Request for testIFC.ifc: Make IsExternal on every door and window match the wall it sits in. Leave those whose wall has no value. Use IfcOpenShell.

First a look at what the model holds.

```python
import ifcopenshell
import ifcopenshell.util.element

model = ifcopenshell.open("testIFC.ifc")
print(model.schema)
seen = {}
for e in model.by_type("IfcDoor") + model.by_type("IfcWindow"):
    if not e.FillsVoids:
        continue
    host = e.FillsVoids[0].RelatingOpeningElement.VoidsElements[0].RelatingBuildingElement
    own = ifcopenshell.util.element.get_pset(e, f"Pset_{e.is_a()[3:].removesuffix('StandardCase')}Common", "IsExternal")
    wall = ifcopenshell.util.element.get_pset(host, "Pset_WallCommon", "IsExternal")
    seen[e.is_a(), own, wall] = seen.get((e.is_a(), own, wall), 0) + 1
for (cls, own, wall), count in sorted(seen.items(), key=str):
    print(count, cls, "IsExternal:", own, "| host wall:", wall)
```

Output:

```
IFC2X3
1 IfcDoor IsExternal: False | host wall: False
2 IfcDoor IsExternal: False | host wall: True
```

```python
import ifcopenshell
import ifcopenshell.api.pset
import ifcopenshell.util.element

model = ifcopenshell.open("testIFC.ifc")

count = 0
for ifc_class, pset_name in (("IfcDoor", "Pset_DoorCommon"), ("IfcWindow", "Pset_WindowCommon")):
    for e in model.by_type(ifc_class):
        if not e.FillsVoids:
            continue
        host = e.FillsVoids[0].RelatingOpeningElement.VoidsElements[0].RelatingBuildingElement
        external = ifcopenshell.util.element.get_pset(host, "Pset_WallCommon", "IsExternal")
        if external is None or ifcopenshell.util.element.get_pset(e, pset_name, "IsExternal") == external:
            continue
        pset = ifcopenshell.api.pset.add_pset(model, product=e, name=pset_name)
        ifcopenshell.api.pset.edit_pset(model, pset=pset, properties={"IsExternal": external})
        count += 1

print(count, "updated")

model.write("testIFC_v2.ifc")
```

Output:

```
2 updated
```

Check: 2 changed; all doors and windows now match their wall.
